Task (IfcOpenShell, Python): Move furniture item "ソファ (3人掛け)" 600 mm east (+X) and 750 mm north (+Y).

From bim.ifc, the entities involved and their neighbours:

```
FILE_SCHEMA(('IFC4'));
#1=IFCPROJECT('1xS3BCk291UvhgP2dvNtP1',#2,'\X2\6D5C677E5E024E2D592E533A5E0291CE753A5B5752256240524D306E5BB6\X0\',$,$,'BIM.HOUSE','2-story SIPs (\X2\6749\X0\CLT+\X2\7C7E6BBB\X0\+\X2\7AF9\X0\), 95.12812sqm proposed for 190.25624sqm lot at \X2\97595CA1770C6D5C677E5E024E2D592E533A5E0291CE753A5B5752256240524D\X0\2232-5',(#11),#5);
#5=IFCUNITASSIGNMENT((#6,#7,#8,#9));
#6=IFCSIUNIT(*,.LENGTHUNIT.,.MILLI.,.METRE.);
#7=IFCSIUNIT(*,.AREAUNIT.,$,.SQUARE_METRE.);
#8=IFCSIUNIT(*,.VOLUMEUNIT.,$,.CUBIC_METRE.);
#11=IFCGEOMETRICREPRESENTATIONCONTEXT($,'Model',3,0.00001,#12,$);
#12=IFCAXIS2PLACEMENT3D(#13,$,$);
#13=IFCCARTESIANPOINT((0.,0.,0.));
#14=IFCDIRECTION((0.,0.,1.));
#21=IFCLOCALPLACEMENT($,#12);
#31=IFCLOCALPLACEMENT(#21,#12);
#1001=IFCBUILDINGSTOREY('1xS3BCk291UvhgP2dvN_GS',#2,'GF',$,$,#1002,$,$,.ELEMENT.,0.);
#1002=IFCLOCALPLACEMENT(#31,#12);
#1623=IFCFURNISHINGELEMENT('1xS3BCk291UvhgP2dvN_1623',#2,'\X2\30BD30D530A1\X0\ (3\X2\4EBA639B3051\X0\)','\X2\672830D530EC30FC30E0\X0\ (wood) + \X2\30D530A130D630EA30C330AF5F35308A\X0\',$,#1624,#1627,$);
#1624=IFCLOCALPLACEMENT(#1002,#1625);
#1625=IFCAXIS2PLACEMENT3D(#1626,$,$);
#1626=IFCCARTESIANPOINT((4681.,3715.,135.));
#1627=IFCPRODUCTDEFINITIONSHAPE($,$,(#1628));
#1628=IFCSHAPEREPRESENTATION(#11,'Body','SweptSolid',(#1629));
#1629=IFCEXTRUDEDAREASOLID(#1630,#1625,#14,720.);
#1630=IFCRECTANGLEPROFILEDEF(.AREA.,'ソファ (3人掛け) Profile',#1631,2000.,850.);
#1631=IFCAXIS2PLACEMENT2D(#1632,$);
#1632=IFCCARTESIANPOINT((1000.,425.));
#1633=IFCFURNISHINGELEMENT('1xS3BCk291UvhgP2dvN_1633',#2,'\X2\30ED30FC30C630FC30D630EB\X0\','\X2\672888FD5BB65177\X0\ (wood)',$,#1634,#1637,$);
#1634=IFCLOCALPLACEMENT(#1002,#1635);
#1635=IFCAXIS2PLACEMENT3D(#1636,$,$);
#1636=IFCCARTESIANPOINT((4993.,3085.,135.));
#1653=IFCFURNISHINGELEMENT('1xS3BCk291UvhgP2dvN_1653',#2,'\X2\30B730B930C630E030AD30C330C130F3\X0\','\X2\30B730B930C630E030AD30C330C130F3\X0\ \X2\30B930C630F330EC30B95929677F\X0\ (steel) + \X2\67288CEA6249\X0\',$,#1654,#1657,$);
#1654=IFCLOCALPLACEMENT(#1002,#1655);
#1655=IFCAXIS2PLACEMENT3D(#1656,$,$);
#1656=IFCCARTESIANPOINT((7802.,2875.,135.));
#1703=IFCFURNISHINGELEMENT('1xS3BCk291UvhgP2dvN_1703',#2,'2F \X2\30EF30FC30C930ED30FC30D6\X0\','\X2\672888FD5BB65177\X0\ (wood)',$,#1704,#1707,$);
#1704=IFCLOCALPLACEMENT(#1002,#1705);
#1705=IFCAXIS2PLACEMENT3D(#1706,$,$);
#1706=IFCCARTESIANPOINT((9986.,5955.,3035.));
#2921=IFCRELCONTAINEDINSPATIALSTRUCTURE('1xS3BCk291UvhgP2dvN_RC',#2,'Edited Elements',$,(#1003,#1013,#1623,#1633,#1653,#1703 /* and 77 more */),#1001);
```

```python
import ifcopenshell
import ifcopenshell.api.geometry
import ifcopenshell.util.placement

model = ifcopenshell.open("bim.ifc")

item = model.by_id(1623)
matrix = ifcopenshell.util.placement.get_local_placement(item.ObjectPlacement)
matrix[0, 3] += 600.0
matrix[1, 3] += 750.0
ifcopenshell.api.geometry.edit_object_placement(model, product=item, matrix=matrix, is_si=False)

print(ifcopenshell.util.placement.get_local_placement(item.ObjectPlacement).round(3) + 0.0)

model.write("bim-out.ifc")
```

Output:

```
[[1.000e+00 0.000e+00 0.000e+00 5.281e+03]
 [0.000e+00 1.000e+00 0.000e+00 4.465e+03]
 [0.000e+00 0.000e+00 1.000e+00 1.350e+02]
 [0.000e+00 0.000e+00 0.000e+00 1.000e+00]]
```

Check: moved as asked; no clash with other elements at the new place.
